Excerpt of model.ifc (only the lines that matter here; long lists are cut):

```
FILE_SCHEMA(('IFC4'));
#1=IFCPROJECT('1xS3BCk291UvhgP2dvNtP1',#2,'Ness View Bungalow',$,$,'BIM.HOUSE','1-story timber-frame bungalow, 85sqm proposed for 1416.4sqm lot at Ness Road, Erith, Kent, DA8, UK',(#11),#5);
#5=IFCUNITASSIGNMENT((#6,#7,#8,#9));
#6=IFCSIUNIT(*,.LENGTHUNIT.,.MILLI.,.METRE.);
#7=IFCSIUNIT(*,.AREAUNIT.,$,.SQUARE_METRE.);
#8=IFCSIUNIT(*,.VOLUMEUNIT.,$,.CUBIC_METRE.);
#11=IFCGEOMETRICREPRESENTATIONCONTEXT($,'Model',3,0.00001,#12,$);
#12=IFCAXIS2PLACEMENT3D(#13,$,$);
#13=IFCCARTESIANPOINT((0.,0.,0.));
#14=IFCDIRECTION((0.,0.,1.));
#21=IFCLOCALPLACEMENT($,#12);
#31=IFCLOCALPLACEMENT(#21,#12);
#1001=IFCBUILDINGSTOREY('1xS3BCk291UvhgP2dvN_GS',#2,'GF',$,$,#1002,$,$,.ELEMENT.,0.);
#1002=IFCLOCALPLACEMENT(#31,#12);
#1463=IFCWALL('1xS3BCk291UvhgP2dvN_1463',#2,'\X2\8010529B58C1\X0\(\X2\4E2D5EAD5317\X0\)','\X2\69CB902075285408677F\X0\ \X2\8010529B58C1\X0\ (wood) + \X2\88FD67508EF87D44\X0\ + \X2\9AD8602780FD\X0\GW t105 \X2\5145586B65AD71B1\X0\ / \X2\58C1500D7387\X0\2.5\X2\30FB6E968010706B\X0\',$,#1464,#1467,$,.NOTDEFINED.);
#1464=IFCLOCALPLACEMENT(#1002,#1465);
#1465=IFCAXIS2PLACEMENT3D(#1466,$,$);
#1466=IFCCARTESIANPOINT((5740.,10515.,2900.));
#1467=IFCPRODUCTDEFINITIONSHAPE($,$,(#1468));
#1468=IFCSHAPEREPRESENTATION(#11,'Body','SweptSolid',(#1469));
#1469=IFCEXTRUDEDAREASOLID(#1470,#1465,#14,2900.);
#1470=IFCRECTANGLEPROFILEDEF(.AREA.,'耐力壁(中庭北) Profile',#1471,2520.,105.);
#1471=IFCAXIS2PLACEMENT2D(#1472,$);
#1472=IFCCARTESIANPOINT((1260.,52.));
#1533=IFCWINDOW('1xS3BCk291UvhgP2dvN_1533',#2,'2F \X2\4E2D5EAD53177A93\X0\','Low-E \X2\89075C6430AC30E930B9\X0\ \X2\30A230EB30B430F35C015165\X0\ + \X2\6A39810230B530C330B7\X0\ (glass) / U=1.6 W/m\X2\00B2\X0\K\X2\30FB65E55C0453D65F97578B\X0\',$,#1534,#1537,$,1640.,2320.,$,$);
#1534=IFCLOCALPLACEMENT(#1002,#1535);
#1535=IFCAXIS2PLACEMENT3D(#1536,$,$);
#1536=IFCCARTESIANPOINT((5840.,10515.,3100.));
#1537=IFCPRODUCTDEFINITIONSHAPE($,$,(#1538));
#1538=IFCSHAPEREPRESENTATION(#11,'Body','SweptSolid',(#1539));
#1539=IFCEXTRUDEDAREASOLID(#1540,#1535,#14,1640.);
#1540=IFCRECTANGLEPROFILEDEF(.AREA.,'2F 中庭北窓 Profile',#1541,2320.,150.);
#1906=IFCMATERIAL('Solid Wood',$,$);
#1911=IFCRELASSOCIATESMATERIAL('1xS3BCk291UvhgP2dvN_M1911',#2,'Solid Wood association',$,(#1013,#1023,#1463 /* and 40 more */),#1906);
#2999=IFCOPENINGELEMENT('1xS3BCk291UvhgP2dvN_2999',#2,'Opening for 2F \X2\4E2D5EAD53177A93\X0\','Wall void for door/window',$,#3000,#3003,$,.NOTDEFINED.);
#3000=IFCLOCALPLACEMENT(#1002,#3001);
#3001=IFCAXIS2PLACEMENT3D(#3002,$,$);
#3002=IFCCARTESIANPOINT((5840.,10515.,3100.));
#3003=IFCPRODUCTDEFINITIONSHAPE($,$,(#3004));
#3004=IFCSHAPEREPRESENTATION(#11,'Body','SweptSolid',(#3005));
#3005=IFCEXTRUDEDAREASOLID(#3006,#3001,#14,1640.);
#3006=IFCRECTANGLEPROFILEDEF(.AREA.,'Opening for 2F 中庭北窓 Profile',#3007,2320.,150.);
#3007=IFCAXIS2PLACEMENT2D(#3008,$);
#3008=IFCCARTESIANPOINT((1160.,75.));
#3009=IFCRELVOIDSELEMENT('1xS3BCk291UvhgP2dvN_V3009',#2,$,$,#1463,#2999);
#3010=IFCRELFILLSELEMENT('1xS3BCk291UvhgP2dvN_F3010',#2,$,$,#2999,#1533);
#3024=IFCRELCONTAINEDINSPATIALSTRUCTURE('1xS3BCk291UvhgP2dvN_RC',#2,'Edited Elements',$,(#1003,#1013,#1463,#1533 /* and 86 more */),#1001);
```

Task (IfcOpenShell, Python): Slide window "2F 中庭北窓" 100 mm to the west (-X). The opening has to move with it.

```python
import ifcopenshell
import ifcopenshell.api.geometry
import ifcopenshell.util.placement
import ifcopenshell.util.unit

model = ifcopenshell.open("model.ifc")
unit_scale = ifcopenshell.util.unit.calculate_unit_scale(model)

window = model.by_guid("1xS3BCk291UvhgP2dvN_1533")
opening = window.FillsVoids[0].RelatingOpeningElement
wall = opening.VoidsElements[0].RelatingBuildingElement

wall_matrix = ifcopenshell.util.placement.get_local_placement(wall.ObjectPlacement)
shift = wall_matrix[:3, 0] * -0.1 / unit_scale
before = ifcopenshell.util.placement.get_local_placement(window.ObjectPlacement)[:3, 3].copy()

# The window is not placed relative to its opening, so move both.
for product in (opening, window):
    matrix = ifcopenshell.util.placement.get_local_placement(product.ObjectPlacement)
    matrix[:3, 3] += shift
    ifcopenshell.api.geometry.edit_object_placement(model, product=product, matrix=matrix, is_si=False)

after = ifcopenshell.util.placement.get_local_placement(window.ObjectPlacement)[:3, 3]
print("window moved by", (after - before).round(3) + 0.0)

model.write("model_edited.ifc")
```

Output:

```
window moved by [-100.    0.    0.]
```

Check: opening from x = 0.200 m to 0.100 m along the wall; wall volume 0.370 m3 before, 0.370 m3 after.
